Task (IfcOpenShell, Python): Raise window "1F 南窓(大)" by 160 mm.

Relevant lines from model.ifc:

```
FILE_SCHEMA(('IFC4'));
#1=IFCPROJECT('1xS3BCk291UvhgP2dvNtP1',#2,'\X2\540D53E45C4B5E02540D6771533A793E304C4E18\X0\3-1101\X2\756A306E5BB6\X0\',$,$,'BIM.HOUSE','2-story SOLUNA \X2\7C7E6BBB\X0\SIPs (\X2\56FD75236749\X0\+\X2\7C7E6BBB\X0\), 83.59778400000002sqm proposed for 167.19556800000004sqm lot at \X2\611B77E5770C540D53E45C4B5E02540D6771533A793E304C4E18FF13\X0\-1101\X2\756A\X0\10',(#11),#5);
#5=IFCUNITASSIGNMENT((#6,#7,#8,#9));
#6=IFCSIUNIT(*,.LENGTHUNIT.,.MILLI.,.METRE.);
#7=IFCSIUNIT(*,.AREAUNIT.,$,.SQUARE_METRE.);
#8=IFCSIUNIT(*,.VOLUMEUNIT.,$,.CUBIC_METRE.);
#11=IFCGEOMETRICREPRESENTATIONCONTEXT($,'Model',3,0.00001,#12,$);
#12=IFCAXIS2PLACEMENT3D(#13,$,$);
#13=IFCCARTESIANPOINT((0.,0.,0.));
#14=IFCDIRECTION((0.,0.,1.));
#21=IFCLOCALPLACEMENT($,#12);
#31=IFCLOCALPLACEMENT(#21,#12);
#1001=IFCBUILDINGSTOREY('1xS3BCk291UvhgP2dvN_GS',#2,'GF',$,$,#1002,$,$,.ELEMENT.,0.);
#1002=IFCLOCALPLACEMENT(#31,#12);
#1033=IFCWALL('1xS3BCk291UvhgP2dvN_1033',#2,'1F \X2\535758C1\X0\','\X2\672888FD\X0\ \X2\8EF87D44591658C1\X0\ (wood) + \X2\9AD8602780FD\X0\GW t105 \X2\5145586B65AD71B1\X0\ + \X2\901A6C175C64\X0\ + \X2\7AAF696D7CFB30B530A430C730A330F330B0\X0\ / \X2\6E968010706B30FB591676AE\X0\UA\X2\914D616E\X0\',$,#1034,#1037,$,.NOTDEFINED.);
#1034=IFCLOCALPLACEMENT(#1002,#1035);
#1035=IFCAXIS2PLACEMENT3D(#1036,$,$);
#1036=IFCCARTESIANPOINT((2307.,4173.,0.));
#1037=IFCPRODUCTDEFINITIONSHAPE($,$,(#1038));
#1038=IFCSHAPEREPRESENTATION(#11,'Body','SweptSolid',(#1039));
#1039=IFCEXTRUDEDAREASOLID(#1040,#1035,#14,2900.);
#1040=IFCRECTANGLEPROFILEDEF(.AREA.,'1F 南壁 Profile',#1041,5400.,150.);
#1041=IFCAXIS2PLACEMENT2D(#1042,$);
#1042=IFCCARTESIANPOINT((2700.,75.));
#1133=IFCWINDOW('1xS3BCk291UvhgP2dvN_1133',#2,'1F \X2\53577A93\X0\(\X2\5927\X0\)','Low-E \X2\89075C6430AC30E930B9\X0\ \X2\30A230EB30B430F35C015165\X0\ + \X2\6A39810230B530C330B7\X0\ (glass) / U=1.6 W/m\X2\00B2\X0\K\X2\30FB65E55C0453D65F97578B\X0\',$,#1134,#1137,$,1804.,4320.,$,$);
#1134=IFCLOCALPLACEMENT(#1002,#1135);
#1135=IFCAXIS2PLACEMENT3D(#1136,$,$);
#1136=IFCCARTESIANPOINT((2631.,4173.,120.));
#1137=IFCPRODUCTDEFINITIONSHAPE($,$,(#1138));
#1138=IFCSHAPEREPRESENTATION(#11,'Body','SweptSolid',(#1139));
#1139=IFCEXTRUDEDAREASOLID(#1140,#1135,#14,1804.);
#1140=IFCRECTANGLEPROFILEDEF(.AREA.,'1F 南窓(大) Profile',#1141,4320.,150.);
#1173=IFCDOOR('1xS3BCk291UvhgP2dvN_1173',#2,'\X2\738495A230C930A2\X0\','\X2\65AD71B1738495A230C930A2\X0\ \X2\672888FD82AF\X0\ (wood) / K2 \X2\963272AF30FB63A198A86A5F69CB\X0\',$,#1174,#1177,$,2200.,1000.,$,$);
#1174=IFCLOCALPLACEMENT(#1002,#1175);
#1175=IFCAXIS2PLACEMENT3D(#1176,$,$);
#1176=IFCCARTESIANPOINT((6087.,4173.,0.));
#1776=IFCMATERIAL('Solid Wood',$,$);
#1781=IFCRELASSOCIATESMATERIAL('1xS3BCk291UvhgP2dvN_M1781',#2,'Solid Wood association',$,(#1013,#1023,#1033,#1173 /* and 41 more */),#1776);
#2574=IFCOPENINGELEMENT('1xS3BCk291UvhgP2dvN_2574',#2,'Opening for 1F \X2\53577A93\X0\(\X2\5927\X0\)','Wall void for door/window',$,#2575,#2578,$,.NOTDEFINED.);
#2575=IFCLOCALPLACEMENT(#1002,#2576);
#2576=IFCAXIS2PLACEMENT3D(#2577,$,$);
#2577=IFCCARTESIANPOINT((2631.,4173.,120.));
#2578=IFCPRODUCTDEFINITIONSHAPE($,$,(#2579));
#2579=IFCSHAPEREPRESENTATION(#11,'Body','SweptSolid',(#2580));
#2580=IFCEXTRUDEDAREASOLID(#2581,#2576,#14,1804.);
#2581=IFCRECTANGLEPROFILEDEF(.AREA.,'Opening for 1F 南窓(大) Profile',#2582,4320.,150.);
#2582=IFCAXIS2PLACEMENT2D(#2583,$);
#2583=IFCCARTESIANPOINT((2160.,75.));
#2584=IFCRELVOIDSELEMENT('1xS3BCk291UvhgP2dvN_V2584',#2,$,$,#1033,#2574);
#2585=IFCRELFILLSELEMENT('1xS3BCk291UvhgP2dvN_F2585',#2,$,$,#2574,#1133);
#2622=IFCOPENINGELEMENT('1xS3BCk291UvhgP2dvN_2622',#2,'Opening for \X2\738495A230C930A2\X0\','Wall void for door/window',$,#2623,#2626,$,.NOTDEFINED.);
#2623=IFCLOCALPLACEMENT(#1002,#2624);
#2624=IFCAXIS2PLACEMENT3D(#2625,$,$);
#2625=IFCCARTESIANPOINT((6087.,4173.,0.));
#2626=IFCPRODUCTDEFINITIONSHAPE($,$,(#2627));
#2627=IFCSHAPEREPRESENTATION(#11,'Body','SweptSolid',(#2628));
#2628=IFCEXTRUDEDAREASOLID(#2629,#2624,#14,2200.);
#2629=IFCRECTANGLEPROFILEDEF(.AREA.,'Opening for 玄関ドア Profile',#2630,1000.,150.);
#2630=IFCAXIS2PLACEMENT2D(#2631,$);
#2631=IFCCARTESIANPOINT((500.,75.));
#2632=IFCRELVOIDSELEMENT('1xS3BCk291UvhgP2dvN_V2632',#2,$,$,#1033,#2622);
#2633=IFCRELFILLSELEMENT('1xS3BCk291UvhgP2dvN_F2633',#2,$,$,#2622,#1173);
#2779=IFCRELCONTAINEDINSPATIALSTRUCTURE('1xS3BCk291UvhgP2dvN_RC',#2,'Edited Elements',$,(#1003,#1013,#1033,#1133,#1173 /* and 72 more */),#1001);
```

```python
import numpy as np
import ifcopenshell
import ifcopenshell.api.geometry
import ifcopenshell.util.placement
import ifcopenshell.util.unit

model = ifcopenshell.open("model.ifc")
unit_scale = ifcopenshell.util.unit.calculate_unit_scale(model)

window = model.by_guid("1xS3BCk291UvhgP2dvN_1133")
opening = window.FillsVoids[0].RelatingOpeningElement
dz = 160.0

shift = np.array([0.0, 0.0, dz])
# The window is not placed relative to its opening, so move both.
for product in (opening, window):
    matrix = ifcopenshell.util.placement.get_local_placement(product.ObjectPlacement)
    matrix[:3, 3] += shift
    ifcopenshell.api.geometry.edit_object_placement(model, product=product, matrix=matrix, is_si=False)

print(f"moved by {dz * unit_scale:+.3f} m")

model.write("model-out.ifc")
```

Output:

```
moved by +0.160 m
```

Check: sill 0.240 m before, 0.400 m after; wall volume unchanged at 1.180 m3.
